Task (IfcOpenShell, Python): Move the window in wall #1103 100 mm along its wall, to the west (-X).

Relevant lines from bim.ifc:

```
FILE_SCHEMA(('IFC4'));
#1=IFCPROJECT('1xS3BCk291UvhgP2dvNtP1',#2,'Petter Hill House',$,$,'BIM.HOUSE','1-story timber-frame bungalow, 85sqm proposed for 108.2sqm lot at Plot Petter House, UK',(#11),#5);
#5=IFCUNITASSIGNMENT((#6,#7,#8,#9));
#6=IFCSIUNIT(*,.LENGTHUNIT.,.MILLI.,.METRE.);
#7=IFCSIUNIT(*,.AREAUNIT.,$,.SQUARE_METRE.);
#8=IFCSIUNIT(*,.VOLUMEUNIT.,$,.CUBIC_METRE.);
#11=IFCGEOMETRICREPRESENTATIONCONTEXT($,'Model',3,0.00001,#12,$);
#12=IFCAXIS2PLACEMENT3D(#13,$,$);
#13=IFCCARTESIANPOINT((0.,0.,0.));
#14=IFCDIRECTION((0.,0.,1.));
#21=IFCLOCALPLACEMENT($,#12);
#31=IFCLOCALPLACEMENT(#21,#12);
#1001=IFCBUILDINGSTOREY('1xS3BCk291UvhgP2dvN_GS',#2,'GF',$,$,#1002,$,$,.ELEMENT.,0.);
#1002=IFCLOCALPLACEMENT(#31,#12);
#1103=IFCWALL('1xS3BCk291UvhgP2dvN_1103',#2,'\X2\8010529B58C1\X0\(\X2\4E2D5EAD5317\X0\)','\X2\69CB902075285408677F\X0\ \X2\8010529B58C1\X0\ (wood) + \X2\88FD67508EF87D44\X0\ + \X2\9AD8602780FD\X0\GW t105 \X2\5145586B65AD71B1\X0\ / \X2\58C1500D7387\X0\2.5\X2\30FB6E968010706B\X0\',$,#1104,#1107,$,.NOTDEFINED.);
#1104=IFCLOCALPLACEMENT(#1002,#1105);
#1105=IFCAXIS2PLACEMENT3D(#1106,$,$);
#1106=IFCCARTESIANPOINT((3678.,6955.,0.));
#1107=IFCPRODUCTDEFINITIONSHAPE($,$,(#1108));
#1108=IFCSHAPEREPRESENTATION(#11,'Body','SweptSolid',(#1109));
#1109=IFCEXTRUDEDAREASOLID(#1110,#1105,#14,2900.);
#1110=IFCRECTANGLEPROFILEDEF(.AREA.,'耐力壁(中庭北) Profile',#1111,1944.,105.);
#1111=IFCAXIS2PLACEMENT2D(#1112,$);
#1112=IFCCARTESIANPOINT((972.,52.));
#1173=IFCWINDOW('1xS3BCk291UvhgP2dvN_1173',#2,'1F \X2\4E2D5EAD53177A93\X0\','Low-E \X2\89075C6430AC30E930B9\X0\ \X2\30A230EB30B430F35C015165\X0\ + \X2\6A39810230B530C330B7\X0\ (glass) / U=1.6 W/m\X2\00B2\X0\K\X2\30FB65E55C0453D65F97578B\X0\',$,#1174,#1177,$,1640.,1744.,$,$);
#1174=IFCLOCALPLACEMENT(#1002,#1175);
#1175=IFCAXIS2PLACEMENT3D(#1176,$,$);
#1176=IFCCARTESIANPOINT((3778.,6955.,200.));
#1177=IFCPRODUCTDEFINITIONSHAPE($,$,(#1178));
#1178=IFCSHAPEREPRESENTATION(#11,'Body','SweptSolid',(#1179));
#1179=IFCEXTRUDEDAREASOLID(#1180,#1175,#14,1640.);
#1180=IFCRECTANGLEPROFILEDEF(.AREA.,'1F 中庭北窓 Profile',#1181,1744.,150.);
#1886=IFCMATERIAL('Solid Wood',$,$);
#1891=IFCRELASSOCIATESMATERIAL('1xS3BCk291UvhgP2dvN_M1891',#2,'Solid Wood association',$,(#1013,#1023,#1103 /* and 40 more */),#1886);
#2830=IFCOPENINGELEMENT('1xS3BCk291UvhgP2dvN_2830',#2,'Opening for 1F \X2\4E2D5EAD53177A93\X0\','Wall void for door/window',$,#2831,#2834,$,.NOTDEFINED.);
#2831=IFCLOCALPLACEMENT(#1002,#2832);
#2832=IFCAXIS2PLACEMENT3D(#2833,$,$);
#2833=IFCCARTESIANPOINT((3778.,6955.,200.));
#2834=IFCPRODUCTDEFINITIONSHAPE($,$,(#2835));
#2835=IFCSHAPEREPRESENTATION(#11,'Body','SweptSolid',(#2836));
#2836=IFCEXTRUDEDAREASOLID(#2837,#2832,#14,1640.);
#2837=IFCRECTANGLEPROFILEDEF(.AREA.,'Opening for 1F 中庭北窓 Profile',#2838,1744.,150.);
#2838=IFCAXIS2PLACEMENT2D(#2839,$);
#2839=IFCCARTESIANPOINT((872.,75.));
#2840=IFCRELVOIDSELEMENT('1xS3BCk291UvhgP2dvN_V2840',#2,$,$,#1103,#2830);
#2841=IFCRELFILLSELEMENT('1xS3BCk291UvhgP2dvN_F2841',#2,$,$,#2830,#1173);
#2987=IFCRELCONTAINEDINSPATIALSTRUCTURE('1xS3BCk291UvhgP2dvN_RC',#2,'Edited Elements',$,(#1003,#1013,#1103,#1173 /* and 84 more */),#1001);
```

```python
import ifcopenshell
import ifcopenshell.api.geometry
import ifcopenshell.util.placement
import ifcopenshell.util.unit

model = ifcopenshell.open("bim.ifc")
unit_scale = ifcopenshell.util.unit.calculate_unit_scale(model)

window = model.by_guid("1xS3BCk291UvhgP2dvN_1173")
opening = window.FillsVoids[0].RelatingOpeningElement
wall = opening.VoidsElements[0].RelatingBuildingElement

wall_matrix = ifcopenshell.util.placement.get_local_placement(wall.ObjectPlacement)
shift = wall_matrix[:3, 0] * -0.1 / unit_scale
before = ifcopenshell.util.placement.get_local_placement(window.ObjectPlacement)[:3, 3].copy()

# The window is not placed relative to its opening, so move both.
for product in (opening, window):
    matrix = ifcopenshell.util.placement.get_local_placement(product.ObjectPlacement)
    matrix[:3, 3] += shift
    ifcopenshell.api.geometry.edit_object_placement(model, product=product, matrix=matrix, is_si=False)

after = ifcopenshell.util.placement.get_local_placement(window.ObjectPlacement)[:3, 3]
print("window moved by", (after - before).round(3) + 0.0)

model.write("bim_v2.ifc")
```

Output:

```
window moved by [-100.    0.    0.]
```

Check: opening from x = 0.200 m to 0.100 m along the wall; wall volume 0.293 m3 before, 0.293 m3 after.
